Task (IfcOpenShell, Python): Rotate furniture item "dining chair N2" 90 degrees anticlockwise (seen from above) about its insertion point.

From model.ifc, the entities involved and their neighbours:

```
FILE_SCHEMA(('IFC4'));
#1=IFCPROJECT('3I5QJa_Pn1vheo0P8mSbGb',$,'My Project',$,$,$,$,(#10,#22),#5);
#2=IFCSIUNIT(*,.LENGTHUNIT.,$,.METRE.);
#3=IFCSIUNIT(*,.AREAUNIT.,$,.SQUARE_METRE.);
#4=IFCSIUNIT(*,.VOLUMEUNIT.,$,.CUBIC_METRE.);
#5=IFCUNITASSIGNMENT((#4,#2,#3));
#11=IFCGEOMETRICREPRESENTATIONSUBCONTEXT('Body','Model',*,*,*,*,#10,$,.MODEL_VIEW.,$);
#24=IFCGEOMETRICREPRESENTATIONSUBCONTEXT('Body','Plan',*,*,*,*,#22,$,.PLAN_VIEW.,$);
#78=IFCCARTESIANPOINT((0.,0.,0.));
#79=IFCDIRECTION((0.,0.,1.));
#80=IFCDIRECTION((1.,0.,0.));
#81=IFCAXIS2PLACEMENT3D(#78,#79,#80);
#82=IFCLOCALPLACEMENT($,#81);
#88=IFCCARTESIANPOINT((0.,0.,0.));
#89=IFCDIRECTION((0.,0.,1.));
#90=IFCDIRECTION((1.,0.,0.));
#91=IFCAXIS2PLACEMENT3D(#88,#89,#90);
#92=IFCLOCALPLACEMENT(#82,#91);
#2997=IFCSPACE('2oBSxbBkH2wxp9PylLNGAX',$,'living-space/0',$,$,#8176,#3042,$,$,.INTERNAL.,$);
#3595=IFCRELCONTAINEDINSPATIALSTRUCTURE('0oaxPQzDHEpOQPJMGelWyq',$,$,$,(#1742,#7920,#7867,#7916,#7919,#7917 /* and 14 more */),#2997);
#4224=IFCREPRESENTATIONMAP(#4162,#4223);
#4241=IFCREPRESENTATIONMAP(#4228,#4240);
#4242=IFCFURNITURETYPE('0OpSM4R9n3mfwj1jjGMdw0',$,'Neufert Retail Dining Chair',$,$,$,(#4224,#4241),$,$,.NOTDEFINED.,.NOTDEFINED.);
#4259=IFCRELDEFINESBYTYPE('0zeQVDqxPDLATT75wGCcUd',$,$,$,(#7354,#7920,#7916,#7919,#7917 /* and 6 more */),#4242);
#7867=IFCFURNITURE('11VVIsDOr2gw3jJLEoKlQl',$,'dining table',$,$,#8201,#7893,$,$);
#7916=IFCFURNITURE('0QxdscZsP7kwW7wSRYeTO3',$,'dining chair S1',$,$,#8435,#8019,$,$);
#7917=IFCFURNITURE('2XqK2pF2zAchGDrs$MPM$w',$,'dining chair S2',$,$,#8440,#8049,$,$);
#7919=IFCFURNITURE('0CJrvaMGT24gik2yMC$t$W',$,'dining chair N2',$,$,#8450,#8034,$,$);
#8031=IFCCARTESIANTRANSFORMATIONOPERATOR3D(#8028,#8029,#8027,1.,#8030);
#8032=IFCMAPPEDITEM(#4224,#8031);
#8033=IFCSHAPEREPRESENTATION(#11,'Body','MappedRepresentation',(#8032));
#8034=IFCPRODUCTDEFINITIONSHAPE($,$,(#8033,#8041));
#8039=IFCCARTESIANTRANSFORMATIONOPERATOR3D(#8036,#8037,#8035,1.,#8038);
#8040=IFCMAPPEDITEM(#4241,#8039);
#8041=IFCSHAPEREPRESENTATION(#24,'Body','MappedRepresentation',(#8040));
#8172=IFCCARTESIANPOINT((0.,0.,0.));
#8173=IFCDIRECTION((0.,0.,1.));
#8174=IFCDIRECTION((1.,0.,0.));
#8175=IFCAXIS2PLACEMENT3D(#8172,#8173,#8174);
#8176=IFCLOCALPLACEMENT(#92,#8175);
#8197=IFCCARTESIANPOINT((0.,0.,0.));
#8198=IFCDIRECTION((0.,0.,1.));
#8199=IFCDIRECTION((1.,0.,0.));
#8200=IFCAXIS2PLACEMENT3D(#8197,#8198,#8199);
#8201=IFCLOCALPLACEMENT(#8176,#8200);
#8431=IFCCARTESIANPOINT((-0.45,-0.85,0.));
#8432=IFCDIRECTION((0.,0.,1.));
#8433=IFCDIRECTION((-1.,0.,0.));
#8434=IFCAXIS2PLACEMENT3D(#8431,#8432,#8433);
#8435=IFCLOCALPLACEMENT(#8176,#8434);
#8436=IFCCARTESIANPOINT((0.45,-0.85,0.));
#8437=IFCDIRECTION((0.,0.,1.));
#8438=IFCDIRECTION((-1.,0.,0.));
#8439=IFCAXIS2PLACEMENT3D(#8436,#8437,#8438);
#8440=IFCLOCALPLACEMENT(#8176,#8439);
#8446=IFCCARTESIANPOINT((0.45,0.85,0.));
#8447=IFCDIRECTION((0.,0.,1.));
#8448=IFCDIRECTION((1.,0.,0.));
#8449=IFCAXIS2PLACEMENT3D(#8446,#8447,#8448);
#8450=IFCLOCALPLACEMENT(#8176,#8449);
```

```python
import ifcopenshell
import ifcopenshell.api.geometry
import ifcopenshell.util.placement

model = ifcopenshell.open("model.ifc")

item = model.by_guid("0CJrvaMGT24gik2yMC$t$W")
matrix = ifcopenshell.util.placement.get_local_placement(item.ObjectPlacement)
matrix = matrix @ ifcopenshell.util.placement.rotation(90, "Z")
ifcopenshell.api.geometry.edit_object_placement(model, product=item, matrix=matrix, is_si=False)

print(ifcopenshell.util.placement.get_local_placement(item.ObjectPlacement).round(3) + 0.0)

model.write("model_rev.ifc")
```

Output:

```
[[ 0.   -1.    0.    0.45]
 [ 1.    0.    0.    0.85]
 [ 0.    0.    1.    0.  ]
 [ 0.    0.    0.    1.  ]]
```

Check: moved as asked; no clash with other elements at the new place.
